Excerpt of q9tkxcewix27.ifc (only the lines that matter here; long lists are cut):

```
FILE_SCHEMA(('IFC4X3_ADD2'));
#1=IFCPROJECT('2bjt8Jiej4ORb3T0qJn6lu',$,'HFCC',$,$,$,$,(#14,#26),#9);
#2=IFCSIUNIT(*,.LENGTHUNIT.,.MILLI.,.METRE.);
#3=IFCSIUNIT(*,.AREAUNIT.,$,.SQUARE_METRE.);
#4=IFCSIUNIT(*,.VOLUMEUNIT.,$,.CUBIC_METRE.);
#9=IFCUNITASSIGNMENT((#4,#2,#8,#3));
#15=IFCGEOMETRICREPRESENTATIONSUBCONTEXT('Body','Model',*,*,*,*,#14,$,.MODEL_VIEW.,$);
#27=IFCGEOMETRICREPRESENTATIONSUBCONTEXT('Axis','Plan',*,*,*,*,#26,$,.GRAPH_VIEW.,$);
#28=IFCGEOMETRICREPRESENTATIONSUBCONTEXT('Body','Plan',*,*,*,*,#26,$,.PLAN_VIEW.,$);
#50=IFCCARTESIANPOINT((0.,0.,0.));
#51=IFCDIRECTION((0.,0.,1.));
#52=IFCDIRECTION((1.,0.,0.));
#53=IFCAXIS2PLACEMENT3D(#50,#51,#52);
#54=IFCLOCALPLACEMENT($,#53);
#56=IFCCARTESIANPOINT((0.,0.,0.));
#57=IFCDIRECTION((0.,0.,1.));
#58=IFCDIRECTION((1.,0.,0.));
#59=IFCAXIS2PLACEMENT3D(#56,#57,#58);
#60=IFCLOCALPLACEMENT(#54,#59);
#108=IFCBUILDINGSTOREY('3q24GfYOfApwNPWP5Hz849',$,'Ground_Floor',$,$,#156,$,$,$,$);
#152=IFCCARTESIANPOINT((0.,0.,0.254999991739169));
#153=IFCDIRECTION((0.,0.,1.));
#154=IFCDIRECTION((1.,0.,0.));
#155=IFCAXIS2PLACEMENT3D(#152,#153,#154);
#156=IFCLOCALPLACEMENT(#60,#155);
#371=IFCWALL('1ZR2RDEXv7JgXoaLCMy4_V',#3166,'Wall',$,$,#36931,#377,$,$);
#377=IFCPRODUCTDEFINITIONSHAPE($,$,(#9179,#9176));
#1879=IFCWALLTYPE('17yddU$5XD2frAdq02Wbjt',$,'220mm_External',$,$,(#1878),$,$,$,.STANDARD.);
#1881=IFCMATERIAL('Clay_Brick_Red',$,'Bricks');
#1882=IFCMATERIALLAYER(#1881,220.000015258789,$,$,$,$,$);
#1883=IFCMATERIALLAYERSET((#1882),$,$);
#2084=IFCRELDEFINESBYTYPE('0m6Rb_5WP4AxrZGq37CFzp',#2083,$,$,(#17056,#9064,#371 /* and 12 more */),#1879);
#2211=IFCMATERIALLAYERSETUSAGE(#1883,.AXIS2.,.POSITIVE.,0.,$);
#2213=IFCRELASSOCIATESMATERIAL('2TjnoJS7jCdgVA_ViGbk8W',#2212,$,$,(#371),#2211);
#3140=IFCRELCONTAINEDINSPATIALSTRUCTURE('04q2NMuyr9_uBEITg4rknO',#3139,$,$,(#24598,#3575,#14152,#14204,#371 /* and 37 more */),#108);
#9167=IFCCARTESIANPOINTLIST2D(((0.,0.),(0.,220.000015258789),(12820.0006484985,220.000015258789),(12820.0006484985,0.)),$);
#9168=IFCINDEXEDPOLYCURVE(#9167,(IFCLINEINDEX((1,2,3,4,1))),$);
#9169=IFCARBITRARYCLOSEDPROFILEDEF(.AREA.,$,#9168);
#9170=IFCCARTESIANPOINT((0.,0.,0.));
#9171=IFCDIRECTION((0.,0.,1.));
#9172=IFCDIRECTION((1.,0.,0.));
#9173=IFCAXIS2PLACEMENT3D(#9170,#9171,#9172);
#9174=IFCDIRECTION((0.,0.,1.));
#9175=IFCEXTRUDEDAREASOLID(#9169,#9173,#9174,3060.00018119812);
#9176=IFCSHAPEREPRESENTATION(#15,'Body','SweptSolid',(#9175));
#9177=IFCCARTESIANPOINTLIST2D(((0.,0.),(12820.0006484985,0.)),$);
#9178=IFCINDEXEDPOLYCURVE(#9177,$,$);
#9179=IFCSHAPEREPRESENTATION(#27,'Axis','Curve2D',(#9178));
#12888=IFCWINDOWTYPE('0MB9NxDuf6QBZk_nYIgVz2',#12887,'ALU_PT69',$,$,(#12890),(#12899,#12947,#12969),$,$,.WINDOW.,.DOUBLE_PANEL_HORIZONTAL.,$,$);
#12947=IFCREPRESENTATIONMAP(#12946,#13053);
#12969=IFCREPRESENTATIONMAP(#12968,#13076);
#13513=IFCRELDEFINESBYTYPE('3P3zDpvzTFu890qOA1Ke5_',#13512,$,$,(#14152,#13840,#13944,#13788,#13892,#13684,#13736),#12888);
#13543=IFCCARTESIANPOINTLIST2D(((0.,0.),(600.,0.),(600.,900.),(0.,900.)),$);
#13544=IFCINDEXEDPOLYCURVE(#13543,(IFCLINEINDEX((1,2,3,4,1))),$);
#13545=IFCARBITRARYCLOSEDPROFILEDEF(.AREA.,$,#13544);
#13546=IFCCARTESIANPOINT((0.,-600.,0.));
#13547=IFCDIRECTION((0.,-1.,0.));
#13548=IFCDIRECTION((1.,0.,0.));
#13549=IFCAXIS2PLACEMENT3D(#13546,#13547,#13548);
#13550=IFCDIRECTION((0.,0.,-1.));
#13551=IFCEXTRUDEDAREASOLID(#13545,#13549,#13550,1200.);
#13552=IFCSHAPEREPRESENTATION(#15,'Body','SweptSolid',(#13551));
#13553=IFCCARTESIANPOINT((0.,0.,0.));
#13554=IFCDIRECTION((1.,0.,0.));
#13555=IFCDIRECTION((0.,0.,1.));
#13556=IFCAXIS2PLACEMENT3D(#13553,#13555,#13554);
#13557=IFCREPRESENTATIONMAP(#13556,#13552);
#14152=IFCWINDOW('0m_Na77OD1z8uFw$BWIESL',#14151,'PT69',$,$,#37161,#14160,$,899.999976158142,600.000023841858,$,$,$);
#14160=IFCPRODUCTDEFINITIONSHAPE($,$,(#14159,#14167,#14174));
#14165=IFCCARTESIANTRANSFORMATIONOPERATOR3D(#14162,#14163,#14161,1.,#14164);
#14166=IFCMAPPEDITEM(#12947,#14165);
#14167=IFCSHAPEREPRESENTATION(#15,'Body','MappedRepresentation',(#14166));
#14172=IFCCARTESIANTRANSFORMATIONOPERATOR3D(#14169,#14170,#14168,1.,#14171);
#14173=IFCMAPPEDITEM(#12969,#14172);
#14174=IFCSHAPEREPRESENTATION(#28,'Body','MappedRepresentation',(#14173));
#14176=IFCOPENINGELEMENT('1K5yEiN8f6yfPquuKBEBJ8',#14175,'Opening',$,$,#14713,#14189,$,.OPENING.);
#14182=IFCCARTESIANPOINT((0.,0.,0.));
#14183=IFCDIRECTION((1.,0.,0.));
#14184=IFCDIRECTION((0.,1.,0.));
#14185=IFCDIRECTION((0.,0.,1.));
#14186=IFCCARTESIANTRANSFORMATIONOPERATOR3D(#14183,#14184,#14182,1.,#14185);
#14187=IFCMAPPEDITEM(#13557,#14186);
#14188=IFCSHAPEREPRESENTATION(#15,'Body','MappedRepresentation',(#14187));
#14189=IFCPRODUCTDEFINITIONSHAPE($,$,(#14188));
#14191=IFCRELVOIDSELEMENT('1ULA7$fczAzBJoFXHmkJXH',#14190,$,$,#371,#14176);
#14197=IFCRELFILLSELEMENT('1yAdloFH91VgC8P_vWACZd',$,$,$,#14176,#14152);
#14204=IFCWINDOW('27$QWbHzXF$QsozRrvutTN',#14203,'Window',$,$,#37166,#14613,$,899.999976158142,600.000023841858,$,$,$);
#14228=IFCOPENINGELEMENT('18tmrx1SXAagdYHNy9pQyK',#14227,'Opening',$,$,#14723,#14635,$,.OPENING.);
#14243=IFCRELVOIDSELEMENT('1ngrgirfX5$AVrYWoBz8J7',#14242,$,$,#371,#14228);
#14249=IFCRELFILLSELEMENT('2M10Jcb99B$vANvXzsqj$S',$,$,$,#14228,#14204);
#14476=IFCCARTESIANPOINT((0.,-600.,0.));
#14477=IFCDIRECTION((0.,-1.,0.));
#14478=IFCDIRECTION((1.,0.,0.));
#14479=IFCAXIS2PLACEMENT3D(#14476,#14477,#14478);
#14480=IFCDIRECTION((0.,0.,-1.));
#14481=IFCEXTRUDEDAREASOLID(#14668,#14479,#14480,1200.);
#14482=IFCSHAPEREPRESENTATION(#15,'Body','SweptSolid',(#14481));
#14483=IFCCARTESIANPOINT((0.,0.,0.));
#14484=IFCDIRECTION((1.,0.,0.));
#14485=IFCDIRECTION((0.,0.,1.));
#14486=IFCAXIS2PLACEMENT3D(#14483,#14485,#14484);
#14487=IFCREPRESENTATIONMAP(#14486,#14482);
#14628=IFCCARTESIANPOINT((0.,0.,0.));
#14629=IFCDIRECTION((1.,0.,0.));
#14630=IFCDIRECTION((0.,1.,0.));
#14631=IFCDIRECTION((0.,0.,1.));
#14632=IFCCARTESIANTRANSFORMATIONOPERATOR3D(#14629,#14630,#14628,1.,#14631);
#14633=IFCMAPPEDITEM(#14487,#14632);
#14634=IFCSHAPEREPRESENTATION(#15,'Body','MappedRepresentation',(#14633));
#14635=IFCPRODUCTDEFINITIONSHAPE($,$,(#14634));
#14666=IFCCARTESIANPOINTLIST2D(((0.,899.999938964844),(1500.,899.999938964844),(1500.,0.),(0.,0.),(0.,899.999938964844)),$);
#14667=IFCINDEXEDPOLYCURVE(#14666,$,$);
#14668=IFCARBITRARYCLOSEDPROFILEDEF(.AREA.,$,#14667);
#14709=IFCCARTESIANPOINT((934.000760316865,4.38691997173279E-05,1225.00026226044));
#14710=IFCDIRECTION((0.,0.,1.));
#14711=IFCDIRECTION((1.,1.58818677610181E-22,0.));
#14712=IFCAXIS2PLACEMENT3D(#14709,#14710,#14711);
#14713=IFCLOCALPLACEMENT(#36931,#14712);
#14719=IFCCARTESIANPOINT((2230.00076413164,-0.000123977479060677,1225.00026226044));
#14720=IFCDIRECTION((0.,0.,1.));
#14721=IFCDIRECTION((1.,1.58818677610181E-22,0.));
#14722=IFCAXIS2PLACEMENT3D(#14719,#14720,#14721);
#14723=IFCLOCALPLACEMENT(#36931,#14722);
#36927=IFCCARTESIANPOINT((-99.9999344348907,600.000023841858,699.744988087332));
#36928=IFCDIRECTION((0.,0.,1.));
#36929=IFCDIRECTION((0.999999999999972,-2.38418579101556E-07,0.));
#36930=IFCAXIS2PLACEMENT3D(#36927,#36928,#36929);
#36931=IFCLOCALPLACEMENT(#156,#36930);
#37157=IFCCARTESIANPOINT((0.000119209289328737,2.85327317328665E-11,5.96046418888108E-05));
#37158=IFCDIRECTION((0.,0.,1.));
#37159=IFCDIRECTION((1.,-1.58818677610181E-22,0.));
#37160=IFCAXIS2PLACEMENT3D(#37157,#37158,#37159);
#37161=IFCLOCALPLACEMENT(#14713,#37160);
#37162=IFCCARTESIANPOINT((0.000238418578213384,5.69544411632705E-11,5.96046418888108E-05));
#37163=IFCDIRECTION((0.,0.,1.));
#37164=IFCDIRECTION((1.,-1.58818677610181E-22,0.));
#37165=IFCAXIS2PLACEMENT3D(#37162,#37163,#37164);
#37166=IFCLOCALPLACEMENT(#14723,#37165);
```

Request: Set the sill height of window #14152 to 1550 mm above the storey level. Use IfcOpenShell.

```python
import numpy as np
import ifcopenshell
import ifcopenshell.api.geometry
import ifcopenshell.geom
import ifcopenshell.util.element
import ifcopenshell.util.placement
import ifcopenshell.util.shape
import ifcopenshell.util.unit

model = ifcopenshell.open("q9tkxcewix27.ifc")
unit_scale = ifcopenshell.util.unit.calculate_unit_scale(model)

window = model.by_guid("0m_Na77OD1z8uFw$BWIESL")
opening = window.FillsVoids[0].RelatingOpeningElement
storey = ifcopenshell.util.element.get_container(window, ifc_class="IfcBuildingStorey")
level = ifcopenshell.util.placement.get_local_placement(storey.ObjectPlacement)[2, 3]

# The opening's origin need not be at the sill, so measure its lowest point.
shape = ifcopenshell.geom.create_shape(ifcopenshell.geom.settings(), opening)
bottom = ifcopenshell.util.shape.get_shape_bottom_elevation(shape, shape.geometry) / unit_scale
dz = level + 1.55 / unit_scale - bottom

shift = np.array([0.0, 0.0, dz])
# The window is placed relative to its opening, so it follows when the opening moves.
matrix = ifcopenshell.util.placement.get_local_placement(opening.ObjectPlacement)
matrix[:3, 3] += shift
ifcopenshell.api.geometry.edit_object_placement(
    model, product=opening, matrix=matrix, is_si=False, should_transform_children=True
)

print(f"moved by {dz * unit_scale:+.3f} m")

model.write("q9tkxcewix27_rev.ifc")
```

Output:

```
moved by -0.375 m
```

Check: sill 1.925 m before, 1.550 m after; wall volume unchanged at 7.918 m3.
